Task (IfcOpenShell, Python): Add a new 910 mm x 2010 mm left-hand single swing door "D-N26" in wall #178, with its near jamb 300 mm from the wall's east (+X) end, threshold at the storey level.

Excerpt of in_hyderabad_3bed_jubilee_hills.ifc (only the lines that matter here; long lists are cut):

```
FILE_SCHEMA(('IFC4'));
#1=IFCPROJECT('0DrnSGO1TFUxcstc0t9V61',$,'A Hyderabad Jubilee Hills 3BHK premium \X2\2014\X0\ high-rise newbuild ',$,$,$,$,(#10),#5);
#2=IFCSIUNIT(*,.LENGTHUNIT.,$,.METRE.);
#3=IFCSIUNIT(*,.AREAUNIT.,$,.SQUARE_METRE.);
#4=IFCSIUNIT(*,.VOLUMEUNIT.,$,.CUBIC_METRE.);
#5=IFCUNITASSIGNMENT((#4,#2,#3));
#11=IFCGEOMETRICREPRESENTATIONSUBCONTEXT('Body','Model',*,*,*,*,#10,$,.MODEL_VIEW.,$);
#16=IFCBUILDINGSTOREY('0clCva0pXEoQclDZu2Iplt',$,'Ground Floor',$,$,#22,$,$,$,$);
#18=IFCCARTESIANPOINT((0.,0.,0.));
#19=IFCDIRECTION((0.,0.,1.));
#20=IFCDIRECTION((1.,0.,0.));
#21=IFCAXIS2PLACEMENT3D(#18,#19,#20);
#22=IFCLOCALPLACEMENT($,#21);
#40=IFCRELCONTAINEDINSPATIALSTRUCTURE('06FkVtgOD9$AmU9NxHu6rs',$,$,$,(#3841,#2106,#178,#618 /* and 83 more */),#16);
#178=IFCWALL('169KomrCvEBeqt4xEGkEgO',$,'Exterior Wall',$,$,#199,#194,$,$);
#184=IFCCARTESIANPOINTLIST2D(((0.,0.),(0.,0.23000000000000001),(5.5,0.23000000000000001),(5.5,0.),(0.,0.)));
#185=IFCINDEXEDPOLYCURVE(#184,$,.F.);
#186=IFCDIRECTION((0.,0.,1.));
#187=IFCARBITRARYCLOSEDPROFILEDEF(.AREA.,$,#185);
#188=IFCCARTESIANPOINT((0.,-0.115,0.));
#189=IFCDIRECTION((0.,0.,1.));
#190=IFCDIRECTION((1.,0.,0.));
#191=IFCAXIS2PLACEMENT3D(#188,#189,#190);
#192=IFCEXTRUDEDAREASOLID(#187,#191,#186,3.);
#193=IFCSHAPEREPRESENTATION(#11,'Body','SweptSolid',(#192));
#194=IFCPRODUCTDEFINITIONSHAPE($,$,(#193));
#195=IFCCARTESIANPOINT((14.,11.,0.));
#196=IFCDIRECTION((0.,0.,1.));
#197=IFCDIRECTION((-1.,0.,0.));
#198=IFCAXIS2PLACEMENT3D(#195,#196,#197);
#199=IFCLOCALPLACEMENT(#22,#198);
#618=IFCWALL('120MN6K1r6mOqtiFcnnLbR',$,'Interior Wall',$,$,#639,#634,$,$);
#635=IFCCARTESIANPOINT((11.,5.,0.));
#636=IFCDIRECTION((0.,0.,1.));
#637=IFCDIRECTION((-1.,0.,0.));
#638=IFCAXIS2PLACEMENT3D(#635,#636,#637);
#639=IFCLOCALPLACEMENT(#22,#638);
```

```python
import numpy as np
import ifcopenshell
import ifcopenshell.api.feature
import ifcopenshell.api.geometry
import ifcopenshell.api.root
import ifcopenshell.api.spatial
import ifcopenshell.geom
import ifcopenshell.util.element
import ifcopenshell.util.placement
import ifcopenshell.util.representation
import ifcopenshell.util.shape
import ifcopenshell.util.unit

model = ifcopenshell.open("in_hyderabad_3bed_jubilee_hills.ifc")
unit_scale = ifcopenshell.util.unit.calculate_unit_scale(model)
settings = ifcopenshell.geom.settings()


def volume(element):
    """Net volume in cubic metres, openings subtracted."""
    shape = ifcopenshell.geom.create_shape(settings, element)
    return ifcopenshell.util.shape.get_volume(shape.geometry)


wall = model.by_guid("169KomrCvEBeqt4xEGkEgO")
storey = ifcopenshell.util.element.get_container(wall, ifc_class="IfcBuildingStorey")
context = ifcopenshell.util.representation.get_context(model, "Model", "Body", "MODEL_VIEW")
before = volume(wall)

width, height, from_end, sill = 0.91, 2.01, 0.3, 0.0  # metres

# The wall runs along its own X axis, and the end named is its -X end.
wall_shape = ifcopenshell.geom.create_shape(settings, wall)
x, y, z = ifcopenshell.util.shape.get_vertices(wall_shape.geometry).T
start = x.min() + from_end
face, thickness = float(y.min()), float(y.max() - y.min())
wall_matrix = ifcopenshell.util.placement.get_local_placement(wall.ObjectPlacement)
level = ifcopenshell.util.placement.get_local_placement(storey.ObjectPlacement)[2, 3]


def in_wall(x, y):
    """Placement at x, y metres in the wall's axes, at sill height."""
    matrix = wall_matrix.copy()
    matrix[:, 3] = wall_matrix @ np.array([x / unit_scale, y / unit_scale, 0.0, 1.0])
    matrix[2, 3] = level + sill / unit_scale
    return matrix


# Opening: a box that overshoots both wall faces by 50 mm.
opening = ifcopenshell.api.root.create_entity(model, ifc_class="IfcOpeningElement", predefined_type="OPENING")
box = ifcopenshell.api.geometry.add_wall_representation(
    model, context=context, length=width, height=height, thickness=thickness + 0.1
)
ifcopenshell.api.geometry.assign_representation(model, product=opening, representation=box)
ifcopenshell.api.geometry.edit_object_placement(model, product=opening, matrix=in_wall(start, face - 0.05), is_si=False)
ifcopenshell.api.feature.add_feature(model, feature=opening, element=wall)

door = ifcopenshell.api.root.create_entity(model, ifc_class="IfcDoor", name="D-N26", predefined_type="DOOR")
door.OverallWidth, door.OverallHeight = width / unit_scale, height / unit_scale
door.OperationType = "SINGLE_SWING_LEFT"
body = ifcopenshell.api.geometry.add_door_representation(
    model,
    context=context,
    overall_width=door.OverallWidth,
    overall_height=door.OverallHeight,
    operation_type="SINGLE_SWING_LEFT",
    lining_properties={"LiningDepth": thickness / unit_scale, "ThresholdDepth": thickness / unit_scale},
)
ifcopenshell.api.geometry.assign_representation(model, product=door, representation=body)
ifcopenshell.api.spatial.assign_container(model, products=[door], relating_structure=storey)
ifcopenshell.api.feature.add_filling(model, opening=opening, element=door)

# The lining spans the wall, so the door starts at the wall face.
ifcopenshell.api.geometry.edit_object_placement(model, product=door, matrix=in_wall(start, face), is_si=False)

after = volume(wall)

print(f"wall volume {before:.3f} -> {after:.3f} m3")

model.write("in_hyderabad_3bed_jubilee_hills_edited.ifc")
```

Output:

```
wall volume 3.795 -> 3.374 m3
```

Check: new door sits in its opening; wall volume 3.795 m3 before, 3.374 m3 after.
